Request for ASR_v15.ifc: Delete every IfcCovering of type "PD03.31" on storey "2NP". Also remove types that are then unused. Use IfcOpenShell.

First a look at what the model holds.

```python
import ifcopenshell
import ifcopenshell.util.element

model = ifcopenshell.open("ASR_v15.ifc")
print(model.schema)
storey = next(s for s in model.by_type("IfcBuildingStorey") if s.Name == "2NP")
coverings = [e for e in ifcopenshell.util.element.get_decomposition(storey) if e.is_a("IfcCovering")]
seen = {}
for e in coverings:
    element_type = ifcopenshell.util.element.get_type(e)
    name = element_type.Name if element_type not in (None, e) else None
    seen[name] = seen.get(name, 0) + 1
for name, count in sorted(seen.items(), key=str):
    print(count, "x", name)
```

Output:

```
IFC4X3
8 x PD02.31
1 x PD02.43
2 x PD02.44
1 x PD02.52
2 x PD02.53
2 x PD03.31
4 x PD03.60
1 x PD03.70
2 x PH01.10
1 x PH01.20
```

```python
import ifcopenshell
import ifcopenshell.api.root
import ifcopenshell.util.element

model = ifcopenshell.open("ASR_v15.ifc")

storey = next(s for s in model.by_type("IfcBuildingStorey") if s.Name == "2NP")
coverings = [e for e in ifcopenshell.util.element.get_decomposition(storey) if e.is_a("IfcCovering")]
targets = [e for e in coverings if (t := ifcopenshell.util.element.get_type(e)) not in (None, e) and t.Name == "PD03.31"]
types = {ifcopenshell.util.element.get_type(e) for e in targets} - {None, *targets}

for e in targets:
    ifcopenshell.api.root.remove_product(model, product=e)
print(len(targets), "removed")

unused = [t for t in types if not ifcopenshell.util.element.get_types(t)]
for t in unused:
    ifcopenshell.api.root.remove_product(model, product=t)
print(len(unused), "unused types removed")

model.write("ASR_v15_rev.ifc")
```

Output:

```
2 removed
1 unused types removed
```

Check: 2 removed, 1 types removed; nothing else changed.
